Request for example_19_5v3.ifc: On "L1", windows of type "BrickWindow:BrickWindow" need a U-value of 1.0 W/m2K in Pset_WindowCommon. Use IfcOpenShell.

First a look at what the model holds.

```python
import ifcopenshell
import ifcopenshell.util.element

model = ifcopenshell.open("example_19_5v3.ifc")
print(model.schema)
storey = next(s for s in model.by_type("IfcBuildingStorey") if s.Name == "L1")
windows = [e for e in ifcopenshell.util.element.get_decomposition(storey) if e.is_a("IfcWindow")]
seen = {}
for e in windows:
    element_type = ifcopenshell.util.element.get_type(e)
    key = (element_type.Name if element_type != e and element_type else None, ifcopenshell.util.element.get_pset(e, "Pset_WindowCommon", "ThermalTransmittance"))
    seen[key] = seen.get(key, 0) + 1
for (name, value), count in sorted(seen.items(), key=str):
    print(count, "x", name, "|", value)
```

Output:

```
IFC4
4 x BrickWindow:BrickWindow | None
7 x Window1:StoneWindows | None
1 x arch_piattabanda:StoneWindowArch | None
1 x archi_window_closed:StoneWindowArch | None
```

```python
import ifcopenshell
import ifcopenshell.api.pset
import ifcopenshell.util.element

model = ifcopenshell.open("example_19_5v3.ifc")

storey = next(s for s in model.by_type("IfcBuildingStorey") if s.Name == "L1")
windows = [e for e in ifcopenshell.util.element.get_decomposition(storey) if e.is_a("IfcWindow")]

count = 0
for e in windows:
    element_type = ifcopenshell.util.element.get_type(e)
    if element_type in (None, e) or element_type.Name != "BrickWindow:BrickWindow":
        continue
    # add_pset returns the element's existing set when there is one.
    pset = ifcopenshell.api.pset.add_pset(model, product=e, name="Pset_WindowCommon")
    ifcopenshell.api.pset.edit_pset(model, pset=pset, properties={"ThermalTransmittance": 1.0})
    count += 1

print(count, "windows updated")

model.write("example_19_5v3_v2.ifc")
```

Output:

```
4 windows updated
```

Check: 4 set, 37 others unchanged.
